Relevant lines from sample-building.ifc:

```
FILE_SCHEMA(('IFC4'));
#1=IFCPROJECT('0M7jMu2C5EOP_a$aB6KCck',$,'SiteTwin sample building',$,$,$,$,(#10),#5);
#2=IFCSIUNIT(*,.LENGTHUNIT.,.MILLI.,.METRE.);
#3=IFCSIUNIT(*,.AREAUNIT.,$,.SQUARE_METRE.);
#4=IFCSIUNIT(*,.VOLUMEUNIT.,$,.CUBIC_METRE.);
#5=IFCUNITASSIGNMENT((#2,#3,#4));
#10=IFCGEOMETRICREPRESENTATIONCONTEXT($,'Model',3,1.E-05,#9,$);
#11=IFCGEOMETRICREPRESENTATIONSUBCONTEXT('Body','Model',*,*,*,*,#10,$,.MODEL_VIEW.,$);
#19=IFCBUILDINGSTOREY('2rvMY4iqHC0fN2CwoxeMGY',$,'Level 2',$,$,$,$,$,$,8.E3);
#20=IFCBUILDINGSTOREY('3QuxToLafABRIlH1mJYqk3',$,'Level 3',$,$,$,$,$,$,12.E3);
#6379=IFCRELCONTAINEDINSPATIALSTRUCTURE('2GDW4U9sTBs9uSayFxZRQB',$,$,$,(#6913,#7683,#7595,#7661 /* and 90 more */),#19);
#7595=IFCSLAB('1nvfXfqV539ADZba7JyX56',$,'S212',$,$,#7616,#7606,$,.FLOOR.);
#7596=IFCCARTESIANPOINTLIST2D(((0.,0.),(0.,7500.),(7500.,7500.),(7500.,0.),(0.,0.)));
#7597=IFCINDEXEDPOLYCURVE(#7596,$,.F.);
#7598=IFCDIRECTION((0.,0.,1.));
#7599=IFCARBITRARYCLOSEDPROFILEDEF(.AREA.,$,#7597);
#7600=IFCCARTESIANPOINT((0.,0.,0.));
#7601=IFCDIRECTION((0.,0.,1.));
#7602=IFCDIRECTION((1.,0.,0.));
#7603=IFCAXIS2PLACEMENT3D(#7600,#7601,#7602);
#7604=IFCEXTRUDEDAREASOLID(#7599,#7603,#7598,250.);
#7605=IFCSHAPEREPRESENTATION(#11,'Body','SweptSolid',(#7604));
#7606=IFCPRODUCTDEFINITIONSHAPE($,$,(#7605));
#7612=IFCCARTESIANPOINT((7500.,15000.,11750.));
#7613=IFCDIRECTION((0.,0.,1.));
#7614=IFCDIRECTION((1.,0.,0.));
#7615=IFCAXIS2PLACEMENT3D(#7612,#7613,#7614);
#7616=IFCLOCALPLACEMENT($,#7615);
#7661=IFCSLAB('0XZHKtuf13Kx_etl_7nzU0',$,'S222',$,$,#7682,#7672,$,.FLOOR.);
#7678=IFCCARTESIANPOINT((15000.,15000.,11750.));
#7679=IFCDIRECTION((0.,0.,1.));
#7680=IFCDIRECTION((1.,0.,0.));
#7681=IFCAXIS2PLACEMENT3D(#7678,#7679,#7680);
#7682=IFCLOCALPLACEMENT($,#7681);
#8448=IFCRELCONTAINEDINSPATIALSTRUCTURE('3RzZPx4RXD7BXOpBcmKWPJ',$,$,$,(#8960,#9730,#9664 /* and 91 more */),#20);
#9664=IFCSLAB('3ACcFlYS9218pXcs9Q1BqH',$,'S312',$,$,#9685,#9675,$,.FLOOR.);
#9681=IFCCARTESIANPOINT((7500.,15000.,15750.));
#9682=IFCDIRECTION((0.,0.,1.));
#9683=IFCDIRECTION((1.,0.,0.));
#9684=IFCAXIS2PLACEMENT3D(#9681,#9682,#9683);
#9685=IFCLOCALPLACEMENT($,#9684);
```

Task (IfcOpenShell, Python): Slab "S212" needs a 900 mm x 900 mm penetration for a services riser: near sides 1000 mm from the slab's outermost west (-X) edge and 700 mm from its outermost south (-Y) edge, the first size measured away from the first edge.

```python
import numpy as np
import ifcopenshell
import ifcopenshell.api.feature
import ifcopenshell.api.geometry
import ifcopenshell.api.root
import ifcopenshell.geom
import ifcopenshell.util.placement
import ifcopenshell.util.representation
import ifcopenshell.util.shape
import ifcopenshell.util.unit

model = ifcopenshell.open("sample-building.ifc")
unit_scale = ifcopenshell.util.unit.calculate_unit_scale(model)
settings = ifcopenshell.geom.settings()


def volume(element):
    """Net volume in cubic metres, openings subtracted."""
    shape = ifcopenshell.geom.create_shape(settings, element)
    return ifcopenshell.util.shape.get_volume(shape.geometry)


slab = model.by_guid("1nvfXfqV539ADZba7JyX56")
before = volume(slab)

# Extent in the slab's own axes, in metres. The edges named are its -X and -Y sides.
slab_shape = ifcopenshell.geom.create_shape(settings, slab)
vertices = ifcopenshell.util.shape.get_vertices(slab_shape.geometry)
x_min, y_min, bottom = vertices.min(axis=0)
top = vertices[:, 2].max()

opening = ifcopenshell.api.root.create_entity(model, ifc_class="IfcOpeningElement", name="Services riser opening", predefined_type="OPENING")
context = ifcopenshell.util.representation.get_context(model, "Model", "Body", "MODEL_VIEW")
width, depth = 0.9, 0.9
outline = [(0.0, 0.0), (width, 0.0), (width, depth), (0.0, depth), (0.0, 0.0)]
# Overshoot both faces by 50 mm so the cut is clean.
shape = ifcopenshell.api.geometry.add_slab_representation(
    model, context=context, depth=top - bottom + 0.1, polyline=outline
)
ifcopenshell.api.geometry.assign_representation(model, product=opening, representation=shape)

matrix = ifcopenshell.util.placement.get_local_placement(slab.ObjectPlacement)
matrix[:, 3] = matrix @ np.append(np.array([x_min + 1, y_min + 0.7, bottom - 0.05]) / unit_scale, 1.0)
ifcopenshell.api.geometry.edit_object_placement(model, product=opening, matrix=matrix, is_si=False)
ifcopenshell.api.feature.add_feature(model, feature=opening, element=slab)

after = volume(slab)

print(f"slab volume {before:.3f} -> {after:.3f} m3")

model.write("sample-building_v2.ifc")
```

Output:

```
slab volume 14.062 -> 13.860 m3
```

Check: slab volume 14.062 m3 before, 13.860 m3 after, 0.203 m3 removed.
